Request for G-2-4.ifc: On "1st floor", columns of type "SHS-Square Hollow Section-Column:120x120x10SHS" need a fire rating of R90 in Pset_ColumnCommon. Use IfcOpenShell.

First a look at what the model holds.

```python
import ifcopenshell
import ifcopenshell.util.element

model = ifcopenshell.open("G-2-4.ifc")
print(model.schema)
storey = next(s for s in model.by_type("IfcBuildingStorey") if s.Name == "1st floor")
columns = [e for e in ifcopenshell.util.element.get_decomposition(storey) if e.is_a("IfcColumn")]
seen = {}
for e in columns:
    element_type = ifcopenshell.util.element.get_type(e)
    key = (element_type.Name if element_type != e and element_type else None, ifcopenshell.util.element.get_pset(e, "Pset_ColumnCommon", "FireRating"))
    seen[key] = seen.get(key, 0) + 1
for (name, value), count in sorted(seen.items(), key=str):
    print(count, "x", name, "|", value)
```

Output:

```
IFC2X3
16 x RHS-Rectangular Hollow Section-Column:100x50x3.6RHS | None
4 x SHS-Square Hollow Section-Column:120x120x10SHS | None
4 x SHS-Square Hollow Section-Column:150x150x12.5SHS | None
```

```python
import ifcopenshell
import ifcopenshell.api.pset
import ifcopenshell.util.element

model = ifcopenshell.open("G-2-4.ifc")

storey = next(s for s in model.by_type("IfcBuildingStorey") if s.Name == "1st floor")
columns = [e for e in ifcopenshell.util.element.get_decomposition(storey) if e.is_a("IfcColumn")]

count = 0
for e in columns:
    element_type = ifcopenshell.util.element.get_type(e)
    if element_type in (None, e) or element_type.Name != "SHS-Square Hollow Section-Column:120x120x10SHS":
        continue
    # add_pset returns the element's existing set when there is one.
    pset = ifcopenshell.api.pset.add_pset(model, product=e, name="Pset_ColumnCommon")
    ifcopenshell.api.pset.edit_pset(model, pset=pset, properties={"FireRating": "R90"})
    count += 1

print(count, "columns updated")

model.write("G-2-4_v2.ifc")
```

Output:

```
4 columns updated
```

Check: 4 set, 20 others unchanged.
